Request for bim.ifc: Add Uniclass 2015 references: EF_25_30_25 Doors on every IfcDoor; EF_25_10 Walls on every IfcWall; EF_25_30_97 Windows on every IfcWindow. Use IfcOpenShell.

First a look at what the model holds.

```python
import ifcopenshell

model = ifcopenshell.open("bim.ifc")
print(model.schema)
print("classifications:", [c.Name for c in model.by_type("IfcClassification")])
for ifc_class in ("IfcDoor", "IfcRoof", "IfcStair", "IfcWall", "IfcWindow"):
    print(ifc_class, len(model.by_type(ifc_class)))
```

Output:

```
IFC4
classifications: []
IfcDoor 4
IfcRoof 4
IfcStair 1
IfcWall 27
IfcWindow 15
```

```python
import ifcopenshell
import ifcopenshell.api.classification

model = ifcopenshell.open("bim.ifc")

system = ifcopenshell.api.classification.add_classification(model, classification="Uniclass 2015")

codes = {
    "IfcDoor": ("EF_25_30_25", "Doors"),
    "IfcWall": ("EF_25_10", "Walls"),
    "IfcWindow": ("EF_25_30_97", "Windows"),
}
for ifc_class, (code, name) in codes.items():
    products = model.by_type(ifc_class)
    ifcopenshell.api.classification.add_reference(
        model, products=products, classification=system, identification=code, name=name
    )
    print(code, len(products))

model.write("bim_rev.ifc")
```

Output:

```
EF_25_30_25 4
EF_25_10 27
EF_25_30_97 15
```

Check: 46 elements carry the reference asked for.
